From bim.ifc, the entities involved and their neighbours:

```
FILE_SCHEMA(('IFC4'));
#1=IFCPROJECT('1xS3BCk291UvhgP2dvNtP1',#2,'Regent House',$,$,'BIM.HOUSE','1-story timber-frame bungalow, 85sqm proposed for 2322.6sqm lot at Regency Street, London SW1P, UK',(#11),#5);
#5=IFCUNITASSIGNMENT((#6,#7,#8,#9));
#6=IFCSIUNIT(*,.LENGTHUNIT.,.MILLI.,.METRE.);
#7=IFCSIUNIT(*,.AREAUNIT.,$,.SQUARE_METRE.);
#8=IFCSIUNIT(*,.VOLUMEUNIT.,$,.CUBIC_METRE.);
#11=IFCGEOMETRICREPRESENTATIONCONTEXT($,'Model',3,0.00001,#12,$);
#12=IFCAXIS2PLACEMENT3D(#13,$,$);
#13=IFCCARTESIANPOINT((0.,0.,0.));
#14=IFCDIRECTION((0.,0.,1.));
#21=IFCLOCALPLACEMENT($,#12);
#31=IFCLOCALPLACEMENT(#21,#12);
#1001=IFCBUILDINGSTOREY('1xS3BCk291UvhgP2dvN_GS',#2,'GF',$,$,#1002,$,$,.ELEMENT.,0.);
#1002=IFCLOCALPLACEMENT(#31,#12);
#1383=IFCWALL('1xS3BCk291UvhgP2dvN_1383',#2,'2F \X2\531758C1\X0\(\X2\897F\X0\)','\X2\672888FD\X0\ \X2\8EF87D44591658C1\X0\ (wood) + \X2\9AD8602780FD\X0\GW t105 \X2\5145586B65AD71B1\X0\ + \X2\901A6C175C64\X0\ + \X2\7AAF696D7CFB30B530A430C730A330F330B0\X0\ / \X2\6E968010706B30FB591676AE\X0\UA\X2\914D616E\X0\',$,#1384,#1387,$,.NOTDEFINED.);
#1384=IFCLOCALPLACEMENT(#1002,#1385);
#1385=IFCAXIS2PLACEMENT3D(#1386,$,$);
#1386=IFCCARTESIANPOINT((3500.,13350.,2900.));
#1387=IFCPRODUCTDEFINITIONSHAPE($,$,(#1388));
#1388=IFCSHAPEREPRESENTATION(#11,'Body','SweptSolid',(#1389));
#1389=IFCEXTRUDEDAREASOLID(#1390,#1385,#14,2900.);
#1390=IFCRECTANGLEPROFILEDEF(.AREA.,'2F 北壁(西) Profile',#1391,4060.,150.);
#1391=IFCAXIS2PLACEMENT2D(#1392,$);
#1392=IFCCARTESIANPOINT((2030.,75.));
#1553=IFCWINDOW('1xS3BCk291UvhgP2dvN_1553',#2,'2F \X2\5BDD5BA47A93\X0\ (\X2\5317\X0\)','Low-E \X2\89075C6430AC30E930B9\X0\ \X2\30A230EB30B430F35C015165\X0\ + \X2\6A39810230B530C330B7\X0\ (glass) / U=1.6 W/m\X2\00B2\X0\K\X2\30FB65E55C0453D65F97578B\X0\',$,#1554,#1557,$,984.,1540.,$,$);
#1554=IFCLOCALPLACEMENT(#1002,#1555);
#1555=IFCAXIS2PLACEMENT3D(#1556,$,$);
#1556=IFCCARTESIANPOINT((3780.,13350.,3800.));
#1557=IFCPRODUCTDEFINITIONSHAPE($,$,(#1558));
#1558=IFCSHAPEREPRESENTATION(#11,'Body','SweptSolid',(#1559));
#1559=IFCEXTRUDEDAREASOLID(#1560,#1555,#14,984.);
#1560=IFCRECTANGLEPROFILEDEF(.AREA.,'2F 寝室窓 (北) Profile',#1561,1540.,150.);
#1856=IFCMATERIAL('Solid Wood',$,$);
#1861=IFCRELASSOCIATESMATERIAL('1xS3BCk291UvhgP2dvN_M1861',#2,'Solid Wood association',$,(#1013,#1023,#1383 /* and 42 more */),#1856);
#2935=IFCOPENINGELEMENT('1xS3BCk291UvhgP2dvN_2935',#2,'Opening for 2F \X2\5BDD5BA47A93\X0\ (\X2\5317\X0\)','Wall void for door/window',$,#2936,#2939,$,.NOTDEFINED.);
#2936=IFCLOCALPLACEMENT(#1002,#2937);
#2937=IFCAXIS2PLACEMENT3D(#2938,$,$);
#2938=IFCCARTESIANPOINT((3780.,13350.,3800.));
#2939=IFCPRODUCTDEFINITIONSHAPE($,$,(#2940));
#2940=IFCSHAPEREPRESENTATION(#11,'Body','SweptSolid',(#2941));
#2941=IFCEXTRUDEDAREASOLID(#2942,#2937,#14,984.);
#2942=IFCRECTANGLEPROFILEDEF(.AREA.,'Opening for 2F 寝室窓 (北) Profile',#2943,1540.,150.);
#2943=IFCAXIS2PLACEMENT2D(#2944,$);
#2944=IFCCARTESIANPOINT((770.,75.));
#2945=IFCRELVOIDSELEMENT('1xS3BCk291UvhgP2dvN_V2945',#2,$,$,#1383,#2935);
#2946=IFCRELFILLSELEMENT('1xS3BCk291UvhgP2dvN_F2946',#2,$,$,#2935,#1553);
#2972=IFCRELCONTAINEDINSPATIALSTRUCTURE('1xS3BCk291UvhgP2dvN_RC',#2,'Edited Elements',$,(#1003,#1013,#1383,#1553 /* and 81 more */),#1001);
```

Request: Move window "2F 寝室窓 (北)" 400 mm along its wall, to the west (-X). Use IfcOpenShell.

```python
import ifcopenshell
import ifcopenshell.api.geometry
import ifcopenshell.util.placement
import ifcopenshell.util.unit

model = ifcopenshell.open("bim.ifc")
unit_scale = ifcopenshell.util.unit.calculate_unit_scale(model)

window = model.by_guid("1xS3BCk291UvhgP2dvN_1553")
opening = window.FillsVoids[0].RelatingOpeningElement
wall = opening.VoidsElements[0].RelatingBuildingElement

wall_matrix = ifcopenshell.util.placement.get_local_placement(wall.ObjectPlacement)
shift = wall_matrix[:3, 0] * -0.4 / unit_scale
before = ifcopenshell.util.placement.get_local_placement(window.ObjectPlacement)[:3, 3].copy()

# The window is not placed relative to its opening, so move both.
for product in (opening, window):
    matrix = ifcopenshell.util.placement.get_local_placement(product.ObjectPlacement)
    matrix[:3, 3] += shift
    ifcopenshell.api.geometry.edit_object_placement(model, product=product, matrix=matrix, is_si=False)

after = ifcopenshell.util.placement.get_local_placement(window.ObjectPlacement)[:3, 3]
print("window moved by", (after - before).round(3) + 0.0)

model.write("bim_edited.ifc")
```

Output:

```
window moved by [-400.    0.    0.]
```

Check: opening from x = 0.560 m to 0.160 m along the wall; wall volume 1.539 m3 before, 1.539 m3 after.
